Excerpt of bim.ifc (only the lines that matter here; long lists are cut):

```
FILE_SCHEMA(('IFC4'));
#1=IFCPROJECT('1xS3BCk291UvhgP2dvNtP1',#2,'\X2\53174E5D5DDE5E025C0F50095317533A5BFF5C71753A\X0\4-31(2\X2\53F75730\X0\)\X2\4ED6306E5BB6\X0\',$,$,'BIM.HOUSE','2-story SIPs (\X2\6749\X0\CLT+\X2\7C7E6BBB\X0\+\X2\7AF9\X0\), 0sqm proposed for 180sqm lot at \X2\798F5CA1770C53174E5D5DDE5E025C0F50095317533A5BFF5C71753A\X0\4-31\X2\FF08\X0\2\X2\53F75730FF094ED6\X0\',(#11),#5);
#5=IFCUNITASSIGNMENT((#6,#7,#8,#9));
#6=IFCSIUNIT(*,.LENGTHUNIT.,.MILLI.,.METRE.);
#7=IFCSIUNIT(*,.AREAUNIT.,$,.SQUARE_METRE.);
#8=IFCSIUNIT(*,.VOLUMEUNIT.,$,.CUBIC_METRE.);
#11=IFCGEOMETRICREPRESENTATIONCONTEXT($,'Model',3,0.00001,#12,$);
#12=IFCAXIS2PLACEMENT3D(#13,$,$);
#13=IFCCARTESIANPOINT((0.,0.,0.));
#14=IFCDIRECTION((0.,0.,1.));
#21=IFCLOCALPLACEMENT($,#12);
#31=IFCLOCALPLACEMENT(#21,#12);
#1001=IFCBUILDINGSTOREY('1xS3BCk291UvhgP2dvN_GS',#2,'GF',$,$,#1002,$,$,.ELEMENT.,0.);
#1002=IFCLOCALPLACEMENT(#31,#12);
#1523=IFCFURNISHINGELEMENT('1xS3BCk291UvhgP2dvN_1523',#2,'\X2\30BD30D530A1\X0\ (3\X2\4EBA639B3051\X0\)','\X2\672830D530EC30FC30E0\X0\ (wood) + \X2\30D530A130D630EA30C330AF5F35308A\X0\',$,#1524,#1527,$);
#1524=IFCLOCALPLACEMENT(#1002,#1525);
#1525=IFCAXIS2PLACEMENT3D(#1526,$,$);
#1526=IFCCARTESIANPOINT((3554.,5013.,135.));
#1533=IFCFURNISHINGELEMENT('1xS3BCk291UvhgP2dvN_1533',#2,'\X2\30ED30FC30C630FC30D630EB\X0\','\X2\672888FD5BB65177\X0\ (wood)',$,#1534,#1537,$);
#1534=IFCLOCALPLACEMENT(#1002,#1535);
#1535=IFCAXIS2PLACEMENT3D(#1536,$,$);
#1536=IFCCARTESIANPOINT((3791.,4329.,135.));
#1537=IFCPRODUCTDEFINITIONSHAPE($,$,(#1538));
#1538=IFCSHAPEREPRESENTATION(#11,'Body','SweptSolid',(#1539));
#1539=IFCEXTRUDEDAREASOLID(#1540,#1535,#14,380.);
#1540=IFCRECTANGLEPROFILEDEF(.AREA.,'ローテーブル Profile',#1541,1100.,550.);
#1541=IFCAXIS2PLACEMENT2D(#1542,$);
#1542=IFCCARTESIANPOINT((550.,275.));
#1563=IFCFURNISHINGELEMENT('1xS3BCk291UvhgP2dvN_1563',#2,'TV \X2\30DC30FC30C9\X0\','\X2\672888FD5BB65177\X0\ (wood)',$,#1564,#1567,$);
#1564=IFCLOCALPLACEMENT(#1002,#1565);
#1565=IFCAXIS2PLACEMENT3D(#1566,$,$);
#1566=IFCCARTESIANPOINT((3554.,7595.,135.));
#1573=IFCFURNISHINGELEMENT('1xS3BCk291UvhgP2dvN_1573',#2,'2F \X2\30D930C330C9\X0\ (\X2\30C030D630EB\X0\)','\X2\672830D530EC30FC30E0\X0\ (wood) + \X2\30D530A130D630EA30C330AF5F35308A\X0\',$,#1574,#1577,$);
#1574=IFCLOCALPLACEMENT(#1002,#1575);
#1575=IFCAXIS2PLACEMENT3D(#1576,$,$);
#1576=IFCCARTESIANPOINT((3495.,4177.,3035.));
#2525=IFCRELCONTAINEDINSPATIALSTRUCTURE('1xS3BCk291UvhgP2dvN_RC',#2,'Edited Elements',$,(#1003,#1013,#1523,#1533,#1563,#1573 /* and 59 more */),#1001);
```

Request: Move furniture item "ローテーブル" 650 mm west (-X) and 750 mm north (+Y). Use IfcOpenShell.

```python
import ifcopenshell
import ifcopenshell.api.geometry
import ifcopenshell.util.placement
import ifcopenshell.util.unit

model = ifcopenshell.open("bim.ifc")
unit_scale = ifcopenshell.util.unit.calculate_unit_scale(model)

item = model.by_guid("1xS3BCk291UvhgP2dvN_1533")
matrix = ifcopenshell.util.placement.get_local_placement(item.ObjectPlacement)
matrix[0, 3] -= 0.65 / unit_scale
matrix[1, 3] += 0.75 / unit_scale
ifcopenshell.api.geometry.edit_object_placement(model, product=item, matrix=matrix, is_si=False)

print(ifcopenshell.util.placement.get_local_placement(item.ObjectPlacement).round(3) + 0.0)

model.write("bim_edited.ifc")
```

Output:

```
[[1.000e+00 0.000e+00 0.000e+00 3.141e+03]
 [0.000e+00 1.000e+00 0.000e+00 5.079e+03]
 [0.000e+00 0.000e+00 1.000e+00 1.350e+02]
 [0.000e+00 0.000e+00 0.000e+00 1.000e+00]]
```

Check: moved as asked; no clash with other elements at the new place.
